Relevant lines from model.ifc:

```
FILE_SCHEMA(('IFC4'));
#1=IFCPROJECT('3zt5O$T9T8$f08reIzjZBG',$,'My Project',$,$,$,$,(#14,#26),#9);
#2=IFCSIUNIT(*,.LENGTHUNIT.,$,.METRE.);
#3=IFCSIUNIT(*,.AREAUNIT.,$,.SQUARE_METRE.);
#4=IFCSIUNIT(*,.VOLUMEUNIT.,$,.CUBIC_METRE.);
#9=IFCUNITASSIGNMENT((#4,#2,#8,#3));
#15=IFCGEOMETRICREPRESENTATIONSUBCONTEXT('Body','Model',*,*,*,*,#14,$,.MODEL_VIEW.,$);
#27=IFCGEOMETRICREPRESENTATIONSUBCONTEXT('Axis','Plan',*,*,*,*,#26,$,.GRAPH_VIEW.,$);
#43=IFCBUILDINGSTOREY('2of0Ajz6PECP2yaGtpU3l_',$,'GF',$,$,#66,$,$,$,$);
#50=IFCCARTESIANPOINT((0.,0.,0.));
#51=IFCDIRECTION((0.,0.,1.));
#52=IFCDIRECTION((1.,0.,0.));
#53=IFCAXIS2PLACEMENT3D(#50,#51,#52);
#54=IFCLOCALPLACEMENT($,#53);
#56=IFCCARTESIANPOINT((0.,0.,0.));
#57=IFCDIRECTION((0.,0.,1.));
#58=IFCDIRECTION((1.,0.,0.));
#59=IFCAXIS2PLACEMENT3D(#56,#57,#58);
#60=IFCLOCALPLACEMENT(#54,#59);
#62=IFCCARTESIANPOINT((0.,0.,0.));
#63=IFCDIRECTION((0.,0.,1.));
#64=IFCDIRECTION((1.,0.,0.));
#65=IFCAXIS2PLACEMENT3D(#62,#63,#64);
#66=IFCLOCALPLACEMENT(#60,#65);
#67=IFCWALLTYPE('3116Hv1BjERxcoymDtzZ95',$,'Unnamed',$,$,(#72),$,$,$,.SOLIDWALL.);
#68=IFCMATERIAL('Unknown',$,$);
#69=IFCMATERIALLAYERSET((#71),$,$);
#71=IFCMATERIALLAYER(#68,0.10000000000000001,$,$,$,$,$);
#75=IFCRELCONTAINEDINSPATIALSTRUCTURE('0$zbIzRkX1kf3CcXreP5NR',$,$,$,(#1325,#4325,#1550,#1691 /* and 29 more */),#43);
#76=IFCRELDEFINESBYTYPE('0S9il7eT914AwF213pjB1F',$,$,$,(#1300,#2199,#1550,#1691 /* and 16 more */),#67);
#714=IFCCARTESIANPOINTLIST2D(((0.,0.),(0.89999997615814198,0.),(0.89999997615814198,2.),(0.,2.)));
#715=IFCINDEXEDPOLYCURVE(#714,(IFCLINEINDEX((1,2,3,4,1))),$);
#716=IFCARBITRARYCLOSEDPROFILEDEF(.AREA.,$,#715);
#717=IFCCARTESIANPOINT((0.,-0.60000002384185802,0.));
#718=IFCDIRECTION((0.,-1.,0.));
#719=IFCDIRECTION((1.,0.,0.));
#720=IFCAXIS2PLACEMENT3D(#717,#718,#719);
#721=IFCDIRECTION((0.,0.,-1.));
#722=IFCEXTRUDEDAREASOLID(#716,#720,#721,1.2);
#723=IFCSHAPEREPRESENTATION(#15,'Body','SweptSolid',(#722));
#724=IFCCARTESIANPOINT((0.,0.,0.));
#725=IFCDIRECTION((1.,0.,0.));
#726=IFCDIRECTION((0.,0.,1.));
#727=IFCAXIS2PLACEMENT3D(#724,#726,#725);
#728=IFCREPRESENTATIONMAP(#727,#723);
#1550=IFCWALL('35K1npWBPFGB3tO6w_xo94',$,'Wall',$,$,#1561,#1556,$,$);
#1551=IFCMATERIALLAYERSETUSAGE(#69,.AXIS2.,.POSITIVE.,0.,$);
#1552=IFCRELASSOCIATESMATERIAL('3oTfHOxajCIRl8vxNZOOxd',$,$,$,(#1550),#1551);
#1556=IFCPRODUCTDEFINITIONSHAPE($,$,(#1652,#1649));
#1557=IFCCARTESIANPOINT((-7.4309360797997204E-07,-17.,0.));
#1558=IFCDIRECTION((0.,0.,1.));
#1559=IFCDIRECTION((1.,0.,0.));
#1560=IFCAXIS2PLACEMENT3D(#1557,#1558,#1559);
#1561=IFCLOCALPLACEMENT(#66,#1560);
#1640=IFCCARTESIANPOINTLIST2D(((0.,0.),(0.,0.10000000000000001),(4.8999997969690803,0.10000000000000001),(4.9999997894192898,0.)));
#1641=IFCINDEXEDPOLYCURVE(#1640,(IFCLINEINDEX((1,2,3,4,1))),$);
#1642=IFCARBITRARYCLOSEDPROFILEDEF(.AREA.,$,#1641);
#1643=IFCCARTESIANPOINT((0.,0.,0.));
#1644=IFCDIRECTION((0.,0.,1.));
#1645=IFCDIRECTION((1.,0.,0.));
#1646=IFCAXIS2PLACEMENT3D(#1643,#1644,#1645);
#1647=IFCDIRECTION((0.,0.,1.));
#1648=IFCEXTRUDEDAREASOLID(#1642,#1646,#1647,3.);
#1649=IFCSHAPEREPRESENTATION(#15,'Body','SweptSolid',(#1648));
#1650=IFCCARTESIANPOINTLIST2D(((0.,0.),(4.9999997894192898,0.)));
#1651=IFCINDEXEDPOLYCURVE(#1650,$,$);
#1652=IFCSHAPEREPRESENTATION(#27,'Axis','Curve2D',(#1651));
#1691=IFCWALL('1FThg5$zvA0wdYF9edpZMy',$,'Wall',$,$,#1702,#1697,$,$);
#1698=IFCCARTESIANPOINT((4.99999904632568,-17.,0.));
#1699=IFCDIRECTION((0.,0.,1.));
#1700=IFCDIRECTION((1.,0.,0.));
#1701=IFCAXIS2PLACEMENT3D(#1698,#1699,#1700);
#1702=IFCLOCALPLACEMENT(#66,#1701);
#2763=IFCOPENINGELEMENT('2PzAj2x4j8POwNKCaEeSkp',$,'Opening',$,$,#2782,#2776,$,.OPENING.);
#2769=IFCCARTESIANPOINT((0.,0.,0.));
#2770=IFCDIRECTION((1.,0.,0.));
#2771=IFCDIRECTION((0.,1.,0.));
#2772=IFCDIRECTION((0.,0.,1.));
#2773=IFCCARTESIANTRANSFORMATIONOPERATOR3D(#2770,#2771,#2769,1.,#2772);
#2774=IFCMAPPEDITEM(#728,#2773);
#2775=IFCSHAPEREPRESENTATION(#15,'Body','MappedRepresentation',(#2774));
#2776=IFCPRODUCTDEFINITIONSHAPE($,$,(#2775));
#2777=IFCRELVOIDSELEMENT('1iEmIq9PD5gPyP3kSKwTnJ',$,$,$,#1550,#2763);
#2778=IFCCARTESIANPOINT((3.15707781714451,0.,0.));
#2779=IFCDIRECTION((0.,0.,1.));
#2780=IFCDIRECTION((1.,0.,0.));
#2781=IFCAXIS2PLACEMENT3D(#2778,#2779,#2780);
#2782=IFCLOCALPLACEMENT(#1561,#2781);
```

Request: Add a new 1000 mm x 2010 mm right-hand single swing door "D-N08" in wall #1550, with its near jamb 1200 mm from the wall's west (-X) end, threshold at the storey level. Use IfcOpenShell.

```python
import numpy as np
import ifcopenshell
import ifcopenshell.api.feature
import ifcopenshell.api.geometry
import ifcopenshell.api.root
import ifcopenshell.api.spatial
import ifcopenshell.geom
import ifcopenshell.util.element
import ifcopenshell.util.placement
import ifcopenshell.util.representation
import ifcopenshell.util.shape
import ifcopenshell.util.unit

model = ifcopenshell.open("model.ifc")
unit_scale = ifcopenshell.util.unit.calculate_unit_scale(model)
settings = ifcopenshell.geom.settings()


def volume(element):
    """Net volume in cubic metres, openings subtracted."""
    shape = ifcopenshell.geom.create_shape(settings, element)
    return ifcopenshell.util.shape.get_volume(shape.geometry)


wall = model.by_id(1550)
storey = ifcopenshell.util.element.get_container(wall, ifc_class="IfcBuildingStorey")
context = ifcopenshell.util.representation.get_context(model, "Model", "Body", "MODEL_VIEW")
before = volume(wall)

width, height, from_end, sill = 1, 2.01, 1.2, 0.0  # metres

# The wall runs along its own X axis, and the end named is its -X end.
wall_shape = ifcopenshell.geom.create_shape(settings, wall)
x, y, z = ifcopenshell.util.shape.get_vertices(wall_shape.geometry).T
start = x.min() + from_end
face, thickness = float(y.min()), float(y.max() - y.min())
wall_matrix = ifcopenshell.util.placement.get_local_placement(wall.ObjectPlacement)
level = ifcopenshell.util.placement.get_local_placement(storey.ObjectPlacement)[2, 3]


def in_wall(x, y):
    """Placement at x, y metres in the wall's axes, at sill height."""
    matrix = wall_matrix.copy()
    matrix[:, 3] = wall_matrix @ np.array([x / unit_scale, y / unit_scale, 0.0, 1.0])
    matrix[2, 3] = level + sill / unit_scale
    return matrix


# Opening: a box that overshoots both wall faces by 50 mm.
opening = ifcopenshell.api.root.create_entity(model, ifc_class="IfcOpeningElement", predefined_type="OPENING")
box = ifcopenshell.api.geometry.add_wall_representation(
    model, context=context, length=width, height=height, thickness=thickness + 0.1
)
ifcopenshell.api.geometry.assign_representation(model, product=opening, representation=box)
ifcopenshell.api.geometry.edit_object_placement(model, product=opening, matrix=in_wall(start, face - 0.05), is_si=False)
ifcopenshell.api.feature.add_feature(model, feature=opening, element=wall)

door = ifcopenshell.api.root.create_entity(model, ifc_class="IfcDoor", name="D-N08", predefined_type="DOOR")
door.OverallWidth, door.OverallHeight = width / unit_scale, height / unit_scale
door.OperationType = "SINGLE_SWING_RIGHT"
body = ifcopenshell.api.geometry.add_door_representation(
    model,
    context=context,
    overall_width=door.OverallWidth,
    overall_height=door.OverallHeight,
    operation_type="SINGLE_SWING_RIGHT",
    lining_properties={"LiningDepth": thickness / unit_scale, "ThresholdDepth": thickness / unit_scale},
)
ifcopenshell.api.geometry.assign_representation(model, product=door, representation=body)
ifcopenshell.api.spatial.assign_container(model, products=[door], relating_structure=storey)
ifcopenshell.api.feature.add_filling(model, opening=opening, element=door)

# The lining spans the wall, so the door starts at the wall face.
ifcopenshell.api.geometry.edit_object_placement(model, product=door, matrix=in_wall(start, face), is_si=False)

after = volume(wall)

print(f"wall volume {before:.3f} -> {after:.3f} m3")

model.write("model_rev.ifc")
```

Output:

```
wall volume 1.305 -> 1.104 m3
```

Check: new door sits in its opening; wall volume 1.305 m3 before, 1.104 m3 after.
